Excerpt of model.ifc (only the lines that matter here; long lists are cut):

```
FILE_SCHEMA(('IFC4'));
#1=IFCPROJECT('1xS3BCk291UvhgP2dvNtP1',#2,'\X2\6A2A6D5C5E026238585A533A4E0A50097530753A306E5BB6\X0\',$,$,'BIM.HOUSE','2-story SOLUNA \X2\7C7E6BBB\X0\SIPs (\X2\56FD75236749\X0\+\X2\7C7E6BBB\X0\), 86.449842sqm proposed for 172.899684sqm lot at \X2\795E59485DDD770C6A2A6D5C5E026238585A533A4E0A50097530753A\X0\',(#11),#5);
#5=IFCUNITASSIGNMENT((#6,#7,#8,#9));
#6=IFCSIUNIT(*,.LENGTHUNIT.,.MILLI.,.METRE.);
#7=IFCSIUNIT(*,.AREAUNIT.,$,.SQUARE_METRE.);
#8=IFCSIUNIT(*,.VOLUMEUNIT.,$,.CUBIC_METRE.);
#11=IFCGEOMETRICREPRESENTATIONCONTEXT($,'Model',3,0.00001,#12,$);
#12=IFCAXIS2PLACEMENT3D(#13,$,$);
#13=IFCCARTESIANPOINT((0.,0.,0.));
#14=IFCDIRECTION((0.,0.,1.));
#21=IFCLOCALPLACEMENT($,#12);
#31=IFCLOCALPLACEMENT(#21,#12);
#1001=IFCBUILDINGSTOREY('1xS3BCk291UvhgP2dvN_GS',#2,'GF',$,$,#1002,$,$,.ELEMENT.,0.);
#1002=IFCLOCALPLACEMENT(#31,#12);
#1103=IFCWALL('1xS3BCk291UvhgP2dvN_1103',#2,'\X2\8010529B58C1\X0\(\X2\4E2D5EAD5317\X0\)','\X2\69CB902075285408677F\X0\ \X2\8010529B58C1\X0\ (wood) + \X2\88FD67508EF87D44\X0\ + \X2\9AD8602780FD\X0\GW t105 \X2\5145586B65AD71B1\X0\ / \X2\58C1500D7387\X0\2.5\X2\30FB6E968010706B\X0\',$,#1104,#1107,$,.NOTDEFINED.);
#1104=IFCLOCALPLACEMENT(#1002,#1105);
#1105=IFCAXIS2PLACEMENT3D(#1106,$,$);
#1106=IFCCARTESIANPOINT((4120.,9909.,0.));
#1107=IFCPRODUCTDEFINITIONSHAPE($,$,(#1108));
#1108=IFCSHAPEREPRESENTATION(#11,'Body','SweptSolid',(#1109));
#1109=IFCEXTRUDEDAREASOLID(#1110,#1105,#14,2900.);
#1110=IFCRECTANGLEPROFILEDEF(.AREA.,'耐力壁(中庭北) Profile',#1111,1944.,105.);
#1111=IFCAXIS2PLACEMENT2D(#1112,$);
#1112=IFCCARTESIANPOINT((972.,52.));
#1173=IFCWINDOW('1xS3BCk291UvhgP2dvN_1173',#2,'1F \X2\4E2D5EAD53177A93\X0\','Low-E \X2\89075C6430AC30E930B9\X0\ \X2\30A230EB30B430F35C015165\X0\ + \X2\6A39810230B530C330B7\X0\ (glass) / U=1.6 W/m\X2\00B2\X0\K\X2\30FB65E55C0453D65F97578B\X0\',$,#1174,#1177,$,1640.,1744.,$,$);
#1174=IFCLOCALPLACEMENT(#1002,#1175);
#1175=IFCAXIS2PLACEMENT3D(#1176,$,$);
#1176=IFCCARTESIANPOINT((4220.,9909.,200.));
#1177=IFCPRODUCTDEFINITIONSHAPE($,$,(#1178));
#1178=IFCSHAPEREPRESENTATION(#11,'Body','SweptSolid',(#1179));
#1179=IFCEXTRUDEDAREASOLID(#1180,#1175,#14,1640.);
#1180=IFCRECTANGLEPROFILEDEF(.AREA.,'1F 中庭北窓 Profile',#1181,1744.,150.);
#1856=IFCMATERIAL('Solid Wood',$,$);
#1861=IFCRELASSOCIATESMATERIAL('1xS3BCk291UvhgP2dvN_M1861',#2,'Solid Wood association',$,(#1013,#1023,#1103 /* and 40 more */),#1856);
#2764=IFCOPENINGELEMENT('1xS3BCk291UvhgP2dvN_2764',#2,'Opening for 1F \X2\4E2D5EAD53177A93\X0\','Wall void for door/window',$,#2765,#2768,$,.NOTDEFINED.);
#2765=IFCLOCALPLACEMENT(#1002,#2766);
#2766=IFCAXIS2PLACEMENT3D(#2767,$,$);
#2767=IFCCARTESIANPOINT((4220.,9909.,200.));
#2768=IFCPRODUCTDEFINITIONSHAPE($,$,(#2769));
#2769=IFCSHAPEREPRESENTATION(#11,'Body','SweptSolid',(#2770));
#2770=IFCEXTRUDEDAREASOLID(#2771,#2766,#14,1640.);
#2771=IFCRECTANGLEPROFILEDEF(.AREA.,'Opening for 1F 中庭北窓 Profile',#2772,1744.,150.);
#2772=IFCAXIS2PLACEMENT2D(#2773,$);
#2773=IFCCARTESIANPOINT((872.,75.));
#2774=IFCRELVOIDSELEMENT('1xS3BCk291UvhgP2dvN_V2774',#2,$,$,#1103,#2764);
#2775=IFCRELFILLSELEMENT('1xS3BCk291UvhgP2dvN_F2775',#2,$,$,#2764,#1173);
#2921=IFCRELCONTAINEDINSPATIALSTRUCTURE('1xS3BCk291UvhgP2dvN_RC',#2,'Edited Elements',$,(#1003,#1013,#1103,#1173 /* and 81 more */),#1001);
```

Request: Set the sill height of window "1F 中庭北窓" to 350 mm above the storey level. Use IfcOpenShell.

```python
import numpy as np
import ifcopenshell
import ifcopenshell.api.geometry
import ifcopenshell.geom
import ifcopenshell.util.element
import ifcopenshell.util.placement
import ifcopenshell.util.shape
import ifcopenshell.util.unit

model = ifcopenshell.open("model.ifc")
unit_scale = ifcopenshell.util.unit.calculate_unit_scale(model)

window = model.by_id(1173)
opening = window.FillsVoids[0].RelatingOpeningElement
storey = ifcopenshell.util.element.get_container(window, ifc_class="IfcBuildingStorey")
level = ifcopenshell.util.placement.get_local_placement(storey.ObjectPlacement)[2, 3]

# The opening's origin need not be at the sill, so measure its lowest point.
shape = ifcopenshell.geom.create_shape(ifcopenshell.geom.settings(), opening)
bottom = ifcopenshell.util.shape.get_shape_bottom_elevation(shape, shape.geometry) / unit_scale
dz = level + 0.35 / unit_scale - bottom

shift = np.array([0.0, 0.0, dz])
# The window is not placed relative to its opening, so move both.
for product in (opening, window):
    matrix = ifcopenshell.util.placement.get_local_placement(product.ObjectPlacement)
    matrix[:3, 3] += shift
    ifcopenshell.api.geometry.edit_object_placement(model, product=product, matrix=matrix, is_si=False)

print(f"moved by {dz * unit_scale:+.3f} m")

model.write("model_v2.ifc")
```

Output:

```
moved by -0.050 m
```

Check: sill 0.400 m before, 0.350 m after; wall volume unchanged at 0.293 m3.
